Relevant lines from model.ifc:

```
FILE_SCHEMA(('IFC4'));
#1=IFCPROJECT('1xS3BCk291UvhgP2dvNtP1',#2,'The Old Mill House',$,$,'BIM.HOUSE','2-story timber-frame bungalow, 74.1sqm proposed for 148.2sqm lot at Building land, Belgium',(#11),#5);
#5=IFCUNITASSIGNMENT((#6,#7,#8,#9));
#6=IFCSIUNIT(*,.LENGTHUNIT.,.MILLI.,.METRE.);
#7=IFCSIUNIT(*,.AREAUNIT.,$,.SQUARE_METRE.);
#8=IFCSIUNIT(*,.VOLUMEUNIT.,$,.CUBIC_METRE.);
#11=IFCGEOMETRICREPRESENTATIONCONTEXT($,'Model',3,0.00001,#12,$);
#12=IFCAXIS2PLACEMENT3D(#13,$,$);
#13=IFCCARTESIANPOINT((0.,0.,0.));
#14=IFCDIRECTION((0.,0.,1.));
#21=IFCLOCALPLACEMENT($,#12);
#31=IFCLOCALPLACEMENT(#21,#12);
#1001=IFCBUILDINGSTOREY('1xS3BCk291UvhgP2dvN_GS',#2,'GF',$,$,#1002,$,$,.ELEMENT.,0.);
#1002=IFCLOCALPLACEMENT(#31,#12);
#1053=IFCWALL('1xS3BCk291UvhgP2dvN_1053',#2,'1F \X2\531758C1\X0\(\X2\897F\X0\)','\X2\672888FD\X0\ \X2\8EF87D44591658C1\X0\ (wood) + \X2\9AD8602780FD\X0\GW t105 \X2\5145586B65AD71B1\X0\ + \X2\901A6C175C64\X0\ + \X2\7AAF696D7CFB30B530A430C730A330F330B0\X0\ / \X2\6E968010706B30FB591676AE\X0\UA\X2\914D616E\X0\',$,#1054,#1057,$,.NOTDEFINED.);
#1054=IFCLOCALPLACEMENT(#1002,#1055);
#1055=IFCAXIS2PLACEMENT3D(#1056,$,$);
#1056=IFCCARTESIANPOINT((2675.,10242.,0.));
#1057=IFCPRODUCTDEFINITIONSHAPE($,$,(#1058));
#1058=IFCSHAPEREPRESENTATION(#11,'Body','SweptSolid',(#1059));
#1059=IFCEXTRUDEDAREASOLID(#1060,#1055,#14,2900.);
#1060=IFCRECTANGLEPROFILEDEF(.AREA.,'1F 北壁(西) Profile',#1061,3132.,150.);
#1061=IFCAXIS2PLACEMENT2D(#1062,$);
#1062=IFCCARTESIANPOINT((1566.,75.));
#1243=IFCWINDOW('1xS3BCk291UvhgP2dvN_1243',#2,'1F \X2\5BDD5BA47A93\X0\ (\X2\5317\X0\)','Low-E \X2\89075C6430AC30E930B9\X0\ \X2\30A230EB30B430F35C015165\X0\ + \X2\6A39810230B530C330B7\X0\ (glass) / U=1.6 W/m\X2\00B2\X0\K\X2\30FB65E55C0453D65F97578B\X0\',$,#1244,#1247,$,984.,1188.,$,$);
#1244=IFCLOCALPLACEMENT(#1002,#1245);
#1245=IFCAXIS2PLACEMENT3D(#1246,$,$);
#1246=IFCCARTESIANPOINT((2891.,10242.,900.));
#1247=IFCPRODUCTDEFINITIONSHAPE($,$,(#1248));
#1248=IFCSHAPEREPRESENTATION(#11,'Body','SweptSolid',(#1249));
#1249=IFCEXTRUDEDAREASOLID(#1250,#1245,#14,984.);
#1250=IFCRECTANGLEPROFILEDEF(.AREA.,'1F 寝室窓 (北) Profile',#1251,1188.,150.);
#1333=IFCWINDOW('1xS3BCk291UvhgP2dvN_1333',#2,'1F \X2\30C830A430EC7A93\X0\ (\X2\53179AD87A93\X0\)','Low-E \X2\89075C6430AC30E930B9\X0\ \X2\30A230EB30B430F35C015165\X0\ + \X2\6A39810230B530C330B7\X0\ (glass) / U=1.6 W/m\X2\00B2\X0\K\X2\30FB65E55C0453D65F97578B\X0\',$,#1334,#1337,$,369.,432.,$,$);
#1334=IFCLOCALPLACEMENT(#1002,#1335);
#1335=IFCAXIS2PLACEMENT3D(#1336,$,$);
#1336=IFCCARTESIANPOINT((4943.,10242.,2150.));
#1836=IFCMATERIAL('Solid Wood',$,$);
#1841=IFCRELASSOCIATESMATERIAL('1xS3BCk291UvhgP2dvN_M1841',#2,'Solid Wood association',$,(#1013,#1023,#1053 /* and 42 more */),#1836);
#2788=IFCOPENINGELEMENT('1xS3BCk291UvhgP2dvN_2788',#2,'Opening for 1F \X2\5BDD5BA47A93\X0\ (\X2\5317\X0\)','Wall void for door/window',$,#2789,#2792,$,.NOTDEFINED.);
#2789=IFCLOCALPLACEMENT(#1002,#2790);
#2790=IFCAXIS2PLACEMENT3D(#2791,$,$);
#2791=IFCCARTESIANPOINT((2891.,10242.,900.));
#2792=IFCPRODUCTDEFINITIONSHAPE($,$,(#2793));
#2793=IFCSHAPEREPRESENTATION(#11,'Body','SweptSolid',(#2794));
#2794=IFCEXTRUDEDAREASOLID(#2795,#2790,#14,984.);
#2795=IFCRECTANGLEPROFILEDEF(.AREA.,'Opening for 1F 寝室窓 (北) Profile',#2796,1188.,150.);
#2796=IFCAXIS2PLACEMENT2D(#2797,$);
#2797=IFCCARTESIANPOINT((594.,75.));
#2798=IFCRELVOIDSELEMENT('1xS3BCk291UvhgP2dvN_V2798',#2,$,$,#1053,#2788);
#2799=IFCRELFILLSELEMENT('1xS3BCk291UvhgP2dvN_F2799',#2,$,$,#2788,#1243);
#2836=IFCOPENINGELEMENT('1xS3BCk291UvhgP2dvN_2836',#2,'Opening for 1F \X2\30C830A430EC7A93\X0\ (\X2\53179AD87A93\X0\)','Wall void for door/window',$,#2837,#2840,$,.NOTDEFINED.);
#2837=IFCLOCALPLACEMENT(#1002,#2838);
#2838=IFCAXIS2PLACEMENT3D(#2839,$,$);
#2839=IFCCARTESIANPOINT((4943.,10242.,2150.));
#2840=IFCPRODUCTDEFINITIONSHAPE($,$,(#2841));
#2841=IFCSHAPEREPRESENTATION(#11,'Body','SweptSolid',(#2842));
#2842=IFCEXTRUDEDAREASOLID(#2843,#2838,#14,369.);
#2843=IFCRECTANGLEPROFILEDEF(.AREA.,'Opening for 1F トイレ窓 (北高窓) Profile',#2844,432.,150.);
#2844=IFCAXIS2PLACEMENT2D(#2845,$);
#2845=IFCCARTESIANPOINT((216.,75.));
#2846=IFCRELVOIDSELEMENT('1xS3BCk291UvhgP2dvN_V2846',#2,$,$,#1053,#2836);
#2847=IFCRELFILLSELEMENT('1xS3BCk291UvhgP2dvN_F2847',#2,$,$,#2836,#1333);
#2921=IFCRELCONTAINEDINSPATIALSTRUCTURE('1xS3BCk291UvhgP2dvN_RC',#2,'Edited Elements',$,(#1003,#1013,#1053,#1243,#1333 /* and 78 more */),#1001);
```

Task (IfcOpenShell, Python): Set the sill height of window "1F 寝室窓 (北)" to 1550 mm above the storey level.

```python
import numpy as np
import ifcopenshell
import ifcopenshell.api.geometry
import ifcopenshell.geom
import ifcopenshell.util.element
import ifcopenshell.util.placement
import ifcopenshell.util.shape
import ifcopenshell.util.unit

model = ifcopenshell.open("model.ifc")
unit_scale = ifcopenshell.util.unit.calculate_unit_scale(model)

window = model.by_guid("1xS3BCk291UvhgP2dvN_1243")
opening = window.FillsVoids[0].RelatingOpeningElement
storey = ifcopenshell.util.element.get_container(window, ifc_class="IfcBuildingStorey")
level = ifcopenshell.util.placement.get_local_placement(storey.ObjectPlacement)[2, 3]

# The opening's origin need not be at the sill, so measure its lowest point.
shape = ifcopenshell.geom.create_shape(ifcopenshell.geom.settings(), opening)
bottom = ifcopenshell.util.shape.get_shape_bottom_elevation(shape, shape.geometry) / unit_scale
dz = level + 1550.0 - bottom

shift = np.array([0.0, 0.0, dz])
# The window is not placed relative to its opening, so move both.
for product in (opening, window):
    matrix = ifcopenshell.util.placement.get_local_placement(product.ObjectPlacement)
    matrix[:3, 3] += shift
    ifcopenshell.api.geometry.edit_object_placement(model, product=product, matrix=matrix, is_si=False)

print(f"moved by {dz * unit_scale:+.3f} m")

model.write("model_updated.ifc")
```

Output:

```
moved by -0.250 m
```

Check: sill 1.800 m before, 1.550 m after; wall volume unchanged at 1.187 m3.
